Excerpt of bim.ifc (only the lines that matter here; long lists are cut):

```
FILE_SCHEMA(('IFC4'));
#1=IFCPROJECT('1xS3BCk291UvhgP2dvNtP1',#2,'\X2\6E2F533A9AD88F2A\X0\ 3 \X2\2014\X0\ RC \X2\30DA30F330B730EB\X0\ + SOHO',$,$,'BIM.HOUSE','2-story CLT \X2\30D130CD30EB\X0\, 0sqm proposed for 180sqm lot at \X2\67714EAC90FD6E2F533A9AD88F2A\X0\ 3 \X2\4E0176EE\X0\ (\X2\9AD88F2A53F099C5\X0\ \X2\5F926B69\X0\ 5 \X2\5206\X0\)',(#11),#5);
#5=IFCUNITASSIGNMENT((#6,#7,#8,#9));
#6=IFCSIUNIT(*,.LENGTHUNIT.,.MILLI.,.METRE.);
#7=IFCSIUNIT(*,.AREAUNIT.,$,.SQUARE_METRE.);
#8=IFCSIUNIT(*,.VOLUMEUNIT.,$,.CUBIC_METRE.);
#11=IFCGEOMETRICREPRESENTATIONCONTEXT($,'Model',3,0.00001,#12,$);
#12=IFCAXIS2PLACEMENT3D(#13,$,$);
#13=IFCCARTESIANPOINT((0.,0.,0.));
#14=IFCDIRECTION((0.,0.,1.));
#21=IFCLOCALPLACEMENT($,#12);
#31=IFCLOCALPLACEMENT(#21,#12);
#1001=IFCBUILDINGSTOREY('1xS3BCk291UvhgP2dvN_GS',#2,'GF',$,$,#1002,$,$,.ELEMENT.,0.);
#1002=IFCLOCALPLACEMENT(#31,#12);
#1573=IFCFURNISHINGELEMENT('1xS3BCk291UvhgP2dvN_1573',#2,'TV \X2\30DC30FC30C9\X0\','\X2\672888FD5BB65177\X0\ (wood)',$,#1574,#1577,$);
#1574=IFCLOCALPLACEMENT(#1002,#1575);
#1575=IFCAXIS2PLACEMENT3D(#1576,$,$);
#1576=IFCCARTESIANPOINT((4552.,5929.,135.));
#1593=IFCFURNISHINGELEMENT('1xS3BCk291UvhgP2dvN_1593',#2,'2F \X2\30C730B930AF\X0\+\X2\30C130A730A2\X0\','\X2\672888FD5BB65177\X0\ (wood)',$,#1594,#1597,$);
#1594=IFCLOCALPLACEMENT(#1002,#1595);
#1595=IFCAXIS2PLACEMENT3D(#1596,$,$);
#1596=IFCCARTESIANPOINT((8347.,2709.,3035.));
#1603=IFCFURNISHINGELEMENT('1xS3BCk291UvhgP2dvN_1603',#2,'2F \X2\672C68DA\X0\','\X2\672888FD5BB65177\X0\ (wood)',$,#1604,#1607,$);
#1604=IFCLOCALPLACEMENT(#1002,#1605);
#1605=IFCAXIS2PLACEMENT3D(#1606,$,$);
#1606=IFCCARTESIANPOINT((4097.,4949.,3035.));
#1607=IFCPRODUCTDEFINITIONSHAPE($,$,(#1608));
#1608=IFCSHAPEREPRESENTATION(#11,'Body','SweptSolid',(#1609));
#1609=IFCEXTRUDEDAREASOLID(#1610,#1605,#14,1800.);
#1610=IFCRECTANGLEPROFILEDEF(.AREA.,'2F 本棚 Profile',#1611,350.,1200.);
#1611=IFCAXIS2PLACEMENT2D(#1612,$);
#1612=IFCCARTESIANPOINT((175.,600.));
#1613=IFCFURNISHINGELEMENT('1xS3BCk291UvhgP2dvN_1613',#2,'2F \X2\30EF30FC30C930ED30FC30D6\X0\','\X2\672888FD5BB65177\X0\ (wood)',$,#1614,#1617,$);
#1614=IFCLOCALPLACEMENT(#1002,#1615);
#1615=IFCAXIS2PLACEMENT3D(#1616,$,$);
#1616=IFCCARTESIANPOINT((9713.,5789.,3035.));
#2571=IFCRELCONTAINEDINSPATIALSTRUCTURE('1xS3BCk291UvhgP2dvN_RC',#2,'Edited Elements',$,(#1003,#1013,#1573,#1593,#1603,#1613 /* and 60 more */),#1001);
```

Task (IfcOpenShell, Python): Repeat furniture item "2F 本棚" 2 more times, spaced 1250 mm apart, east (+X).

```python
import numpy as np
import ifcopenshell
import ifcopenshell.api.geometry
import ifcopenshell.api.root
import ifcopenshell.util.element
import ifcopenshell.util.placement
import ifcopenshell.util.unit

model = ifcopenshell.open("bim.ifc")
unit_scale = ifcopenshell.util.unit.calculate_unit_scale(model)


def reuse_history(source, copy):
    """copy_class also copies each property set's owner history, people and application; keep the originals."""
    for rel in copy.IsDefinedBy:
        if rel.is_a("IfcRelDefinesByProperties") and (history := rel.RelatingPropertyDefinition.OwnerHistory):
            rel.RelatingPropertyDefinition.OwnerHistory = source.OwnerHistory
            ifcopenshell.util.element.remove_deep2(model, history)


source = model.by_guid("1xS3BCk291UvhgP2dvN_1603")
base = ifcopenshell.util.placement.get_local_placement(source.ObjectPlacement)
step = np.array([1.0, 0.0, 0.0]) * 1.25 / unit_scale

for i in range(1, 3):
    copy = ifcopenshell.api.root.copy_class(model, product=source)
    copy.Representation = ifcopenshell.util.element.copy_deep(
        model, source.Representation, exclude=["IfcGeometricRepresentationContext", "IfcRepresentationMap"]
    )
    reuse_history(source, copy)
    matrix = base.copy()
    matrix[:3, 3] += i * step
    print("added at", matrix[:3, 3].round(3) + 0.0)
    ifcopenshell.api.geometry.edit_object_placement(model, product=copy, matrix=matrix, is_si=False)

model.write("bim_edited.ifc")
```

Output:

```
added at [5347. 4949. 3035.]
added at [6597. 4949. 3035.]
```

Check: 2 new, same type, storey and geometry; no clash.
